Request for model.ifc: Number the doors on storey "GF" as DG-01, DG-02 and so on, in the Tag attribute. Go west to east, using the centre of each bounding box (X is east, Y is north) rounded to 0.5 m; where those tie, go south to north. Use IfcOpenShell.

First a look at what the model holds.

```python
import ifcopenshell
import ifcopenshell.util.element
import ifcopenshell.util.placement

model = ifcopenshell.open("model.ifc")
print(model.schema)
storey = next(s for s in model.by_type("IfcBuildingStorey") if s.Name == "GF")
doors = [e for e in ifcopenshell.util.element.get_decomposition(storey) if e.is_a("IfcDoor")]
for e in sorted(doors, key=lambda e: e.id()):
    origin = ifcopenshell.util.placement.get_local_placement(e.ObjectPlacement)[:3, 3]
    print(e.id(), e.Tag, e.Name, origin.round(2) + 0.0, sep=" | ")
```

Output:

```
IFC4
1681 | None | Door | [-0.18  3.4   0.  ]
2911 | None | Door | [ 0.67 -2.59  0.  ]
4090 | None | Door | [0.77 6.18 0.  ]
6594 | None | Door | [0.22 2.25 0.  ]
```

```python
import ifcopenshell
import ifcopenshell.geom
import ifcopenshell.util.element
import ifcopenshell.util.shape

model = ifcopenshell.open("model.ifc")
settings = ifcopenshell.geom.settings()
settings.set("use-world-coords", True)


def centre(element):
    shape = ifcopenshell.geom.create_shape(settings, element)
    return ifcopenshell.util.shape.get_bbox_centroid(shape.geometry)


storey = next(s for s in model.by_type("IfcBuildingStorey") if s.Name == "GF")
doors = [e for e in ifcopenshell.util.element.get_decomposition(storey) if e.is_a("IfcDoor")]

# Insertion points can sit at a corner or the storey origin, so sort by the geometry (in metres).
centres = {e: centre(e) for e in doors}
doors.sort(key=lambda e: (round(centres[e][0] / 0.5), centres[e][1]))

for i, e in enumerate(doors, start=1):
    number = f"DG-{i:02d}"
    e.Tag = number
    print(e.id(), number)

model.write("model_edited.ifc")
```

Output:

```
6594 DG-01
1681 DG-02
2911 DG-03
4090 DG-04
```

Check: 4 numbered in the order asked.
